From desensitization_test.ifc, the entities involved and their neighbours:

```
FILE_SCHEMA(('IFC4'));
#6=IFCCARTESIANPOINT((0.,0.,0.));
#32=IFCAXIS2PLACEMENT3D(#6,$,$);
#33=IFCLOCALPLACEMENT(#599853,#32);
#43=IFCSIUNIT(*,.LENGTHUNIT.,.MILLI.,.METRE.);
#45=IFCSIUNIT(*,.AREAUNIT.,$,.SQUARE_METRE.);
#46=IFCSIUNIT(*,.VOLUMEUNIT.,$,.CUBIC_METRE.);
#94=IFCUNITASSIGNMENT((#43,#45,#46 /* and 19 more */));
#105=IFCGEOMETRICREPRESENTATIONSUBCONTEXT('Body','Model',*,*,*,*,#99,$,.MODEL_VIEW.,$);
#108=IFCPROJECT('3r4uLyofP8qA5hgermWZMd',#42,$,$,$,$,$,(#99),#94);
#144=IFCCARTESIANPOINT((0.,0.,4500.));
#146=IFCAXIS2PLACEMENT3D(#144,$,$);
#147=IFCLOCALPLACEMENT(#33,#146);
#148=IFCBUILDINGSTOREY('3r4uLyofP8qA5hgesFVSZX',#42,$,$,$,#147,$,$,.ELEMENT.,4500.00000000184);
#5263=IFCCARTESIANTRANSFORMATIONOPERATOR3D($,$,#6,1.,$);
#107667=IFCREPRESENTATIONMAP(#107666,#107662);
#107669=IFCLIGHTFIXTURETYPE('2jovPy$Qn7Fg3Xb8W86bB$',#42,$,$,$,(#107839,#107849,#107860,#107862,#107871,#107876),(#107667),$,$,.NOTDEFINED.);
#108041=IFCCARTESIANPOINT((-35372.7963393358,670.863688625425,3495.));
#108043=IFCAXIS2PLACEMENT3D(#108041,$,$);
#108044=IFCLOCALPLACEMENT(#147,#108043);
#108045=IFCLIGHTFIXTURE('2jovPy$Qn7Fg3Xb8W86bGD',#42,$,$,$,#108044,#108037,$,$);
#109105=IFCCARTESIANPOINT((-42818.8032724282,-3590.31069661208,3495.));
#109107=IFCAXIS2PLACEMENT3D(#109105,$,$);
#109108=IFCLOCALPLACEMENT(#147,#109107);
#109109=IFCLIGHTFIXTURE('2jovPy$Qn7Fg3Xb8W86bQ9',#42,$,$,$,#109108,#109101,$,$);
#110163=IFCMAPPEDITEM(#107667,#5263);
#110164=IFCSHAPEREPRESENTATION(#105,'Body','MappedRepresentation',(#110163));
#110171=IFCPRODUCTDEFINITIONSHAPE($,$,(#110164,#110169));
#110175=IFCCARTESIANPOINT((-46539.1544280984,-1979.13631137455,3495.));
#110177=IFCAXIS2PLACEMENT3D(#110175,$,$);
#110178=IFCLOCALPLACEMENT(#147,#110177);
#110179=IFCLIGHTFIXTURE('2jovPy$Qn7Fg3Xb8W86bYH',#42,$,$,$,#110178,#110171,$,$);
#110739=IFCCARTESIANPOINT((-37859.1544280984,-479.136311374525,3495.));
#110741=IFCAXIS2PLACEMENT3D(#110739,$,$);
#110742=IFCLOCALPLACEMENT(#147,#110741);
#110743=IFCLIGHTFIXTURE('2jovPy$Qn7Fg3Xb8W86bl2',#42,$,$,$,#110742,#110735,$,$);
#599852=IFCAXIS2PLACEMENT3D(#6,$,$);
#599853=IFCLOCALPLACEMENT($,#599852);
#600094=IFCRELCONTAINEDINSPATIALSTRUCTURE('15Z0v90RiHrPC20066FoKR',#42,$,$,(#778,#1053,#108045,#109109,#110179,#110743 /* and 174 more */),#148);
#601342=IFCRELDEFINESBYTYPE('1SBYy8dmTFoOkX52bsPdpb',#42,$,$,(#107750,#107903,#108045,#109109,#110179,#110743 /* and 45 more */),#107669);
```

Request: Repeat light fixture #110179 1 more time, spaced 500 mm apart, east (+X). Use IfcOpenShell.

```python
import numpy as np
import ifcopenshell
import ifcopenshell.api.geometry
import ifcopenshell.api.root
import ifcopenshell.util.element
import ifcopenshell.util.placement
import ifcopenshell.util.unit

model = ifcopenshell.open("desensitization_test.ifc")
unit_scale = ifcopenshell.util.unit.calculate_unit_scale(model)


def reuse_history(source, copy):
    """copy_class also copies each property set's owner history, people and application; keep the originals."""
    for rel in copy.IsDefinedBy:
        if rel.is_a("IfcRelDefinesByProperties") and (history := rel.RelatingPropertyDefinition.OwnerHistory):
            rel.RelatingPropertyDefinition.OwnerHistory = source.OwnerHistory
            ifcopenshell.util.element.remove_deep2(model, history)


source = model.by_guid("2jovPy$Qn7Fg3Xb8W86bYH")
base = ifcopenshell.util.placement.get_local_placement(source.ObjectPlacement)
step = np.array([1.0, 0.0, 0.0]) * 0.5 / unit_scale

for i in range(1, 2):
    copy = ifcopenshell.api.root.copy_class(model, product=source)
    copy.Representation = ifcopenshell.util.element.copy_deep(
        model, source.Representation, exclude=["IfcGeometricRepresentationContext", "IfcRepresentationMap"]
    )
    reuse_history(source, copy)
    matrix = base.copy()
    matrix[:3, 3] += i * step
    print("added at", matrix[:3, 3].round(3) + 0.0)
    ifcopenshell.api.geometry.edit_object_placement(model, product=copy, matrix=matrix, is_si=False)

model.write("desensitization_test_edited.ifc")
```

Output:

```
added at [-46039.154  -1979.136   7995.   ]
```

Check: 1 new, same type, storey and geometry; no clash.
